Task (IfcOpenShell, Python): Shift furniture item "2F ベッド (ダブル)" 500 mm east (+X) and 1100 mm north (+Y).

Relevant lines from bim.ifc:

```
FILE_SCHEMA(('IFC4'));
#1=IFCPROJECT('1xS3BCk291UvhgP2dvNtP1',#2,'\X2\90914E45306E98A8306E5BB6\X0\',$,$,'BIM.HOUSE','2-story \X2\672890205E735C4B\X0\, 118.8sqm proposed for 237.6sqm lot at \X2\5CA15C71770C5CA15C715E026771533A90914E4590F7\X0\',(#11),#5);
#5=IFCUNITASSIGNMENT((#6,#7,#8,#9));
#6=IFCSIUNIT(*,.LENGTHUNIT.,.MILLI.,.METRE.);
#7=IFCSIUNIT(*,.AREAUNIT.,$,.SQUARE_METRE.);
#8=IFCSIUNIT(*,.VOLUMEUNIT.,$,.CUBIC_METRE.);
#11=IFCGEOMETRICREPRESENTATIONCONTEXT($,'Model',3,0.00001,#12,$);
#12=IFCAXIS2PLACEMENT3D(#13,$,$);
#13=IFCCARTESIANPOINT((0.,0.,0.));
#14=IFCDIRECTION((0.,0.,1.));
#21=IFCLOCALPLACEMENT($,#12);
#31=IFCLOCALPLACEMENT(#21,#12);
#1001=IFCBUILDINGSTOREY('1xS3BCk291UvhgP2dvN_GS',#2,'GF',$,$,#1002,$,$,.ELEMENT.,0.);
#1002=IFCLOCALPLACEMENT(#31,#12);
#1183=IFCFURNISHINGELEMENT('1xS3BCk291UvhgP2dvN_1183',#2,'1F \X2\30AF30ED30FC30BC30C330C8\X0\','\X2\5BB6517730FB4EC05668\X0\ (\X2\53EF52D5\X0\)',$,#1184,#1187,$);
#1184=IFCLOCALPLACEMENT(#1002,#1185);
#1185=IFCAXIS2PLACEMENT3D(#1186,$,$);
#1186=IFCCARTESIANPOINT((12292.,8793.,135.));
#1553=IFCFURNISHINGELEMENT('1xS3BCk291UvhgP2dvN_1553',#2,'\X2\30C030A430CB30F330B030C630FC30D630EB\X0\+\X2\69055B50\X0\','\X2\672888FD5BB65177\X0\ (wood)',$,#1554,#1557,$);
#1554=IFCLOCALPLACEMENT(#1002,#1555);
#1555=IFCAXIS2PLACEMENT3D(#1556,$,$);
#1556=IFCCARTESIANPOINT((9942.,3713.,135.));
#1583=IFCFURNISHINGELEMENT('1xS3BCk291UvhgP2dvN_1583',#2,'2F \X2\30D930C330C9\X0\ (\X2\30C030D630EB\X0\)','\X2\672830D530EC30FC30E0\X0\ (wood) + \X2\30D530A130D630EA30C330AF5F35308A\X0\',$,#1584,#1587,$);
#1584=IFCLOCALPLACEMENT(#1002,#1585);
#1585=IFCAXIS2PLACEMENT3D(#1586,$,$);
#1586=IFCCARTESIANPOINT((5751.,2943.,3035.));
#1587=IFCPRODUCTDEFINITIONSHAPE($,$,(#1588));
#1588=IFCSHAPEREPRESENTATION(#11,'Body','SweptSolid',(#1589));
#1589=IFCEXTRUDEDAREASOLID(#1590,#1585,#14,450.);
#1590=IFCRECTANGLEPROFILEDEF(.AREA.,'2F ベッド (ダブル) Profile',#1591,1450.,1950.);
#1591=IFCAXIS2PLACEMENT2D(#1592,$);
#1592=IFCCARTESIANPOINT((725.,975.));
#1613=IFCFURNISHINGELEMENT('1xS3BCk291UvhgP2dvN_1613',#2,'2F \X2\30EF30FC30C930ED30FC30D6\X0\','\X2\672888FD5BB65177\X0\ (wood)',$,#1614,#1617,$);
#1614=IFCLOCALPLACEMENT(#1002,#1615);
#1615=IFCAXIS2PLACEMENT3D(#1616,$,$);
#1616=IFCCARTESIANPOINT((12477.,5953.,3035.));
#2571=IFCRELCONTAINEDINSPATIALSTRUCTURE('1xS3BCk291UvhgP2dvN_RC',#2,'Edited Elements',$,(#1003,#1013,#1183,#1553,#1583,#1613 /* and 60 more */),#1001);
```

```python
import ifcopenshell
import ifcopenshell.api.geometry
import ifcopenshell.util.placement
import ifcopenshell.util.unit

model = ifcopenshell.open("bim.ifc")
unit_scale = ifcopenshell.util.unit.calculate_unit_scale(model)

item = model.by_guid("1xS3BCk291UvhgP2dvN_1583")
matrix = ifcopenshell.util.placement.get_local_placement(item.ObjectPlacement)
matrix[0, 3] += 0.5 / unit_scale
matrix[1, 3] += 1.1 / unit_scale
ifcopenshell.api.geometry.edit_object_placement(model, product=item, matrix=matrix, is_si=False)

print(ifcopenshell.util.placement.get_local_placement(item.ObjectPlacement).round(3) + 0.0)

model.write("bim_updated.ifc")
```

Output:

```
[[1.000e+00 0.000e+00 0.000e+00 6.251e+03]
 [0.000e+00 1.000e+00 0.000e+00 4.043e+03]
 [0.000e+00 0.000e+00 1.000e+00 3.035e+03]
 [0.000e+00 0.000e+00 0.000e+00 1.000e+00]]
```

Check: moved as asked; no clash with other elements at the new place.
